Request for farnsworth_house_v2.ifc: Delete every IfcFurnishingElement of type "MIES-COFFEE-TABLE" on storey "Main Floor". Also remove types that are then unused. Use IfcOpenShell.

First a look at what the model holds.

```python
import ifcopenshell
import ifcopenshell.util.element

model = ifcopenshell.open("farnsworth_house_v2.ifc")
print(model.schema)
storey = next(s for s in model.by_type("IfcBuildingStorey") if s.Name == "Main Floor")
furniture = [e for e in ifcopenshell.util.element.get_decomposition(storey) if e.is_a("IfcFurnishingElement")]
seen = {}
for e in furniture:
    element_type = ifcopenshell.util.element.get_type(e)
    name = element_type.Name if element_type not in (None, e) else None
    seen[name] = seen.get(name, 0) + 1
for name, count in sorted(seen.items(), key=str):
    print(count, "x", name)
```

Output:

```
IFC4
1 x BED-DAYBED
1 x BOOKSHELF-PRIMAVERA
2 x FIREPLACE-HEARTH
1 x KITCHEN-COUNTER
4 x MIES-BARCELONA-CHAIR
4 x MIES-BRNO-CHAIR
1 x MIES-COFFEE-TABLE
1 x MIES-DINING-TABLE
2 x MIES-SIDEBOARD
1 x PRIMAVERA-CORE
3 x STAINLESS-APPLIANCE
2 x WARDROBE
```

```python
import ifcopenshell
import ifcopenshell.api.root
import ifcopenshell.util.element

model = ifcopenshell.open("farnsworth_house_v2.ifc")

storey = next(s for s in model.by_type("IfcBuildingStorey") if s.Name == "Main Floor")
furniture = [e for e in ifcopenshell.util.element.get_decomposition(storey) if e.is_a("IfcFurnishingElement")]
targets = [e for e in furniture if (t := ifcopenshell.util.element.get_type(e)) not in (None, e) and t.Name == "MIES-COFFEE-TABLE"]
types = {ifcopenshell.util.element.get_type(e) for e in targets} - {None, *targets}

for e in targets:
    ifcopenshell.api.root.remove_product(model, product=e)
print(len(targets), "removed")

unused = [t for t in types if not ifcopenshell.util.element.get_types(t)]
for t in unused:
    ifcopenshell.api.root.remove_product(model, product=t)
print(len(unused), "unused types removed")

model.write("farnsworth_house_v2_v2.ifc")
```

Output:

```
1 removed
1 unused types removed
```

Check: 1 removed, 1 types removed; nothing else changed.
